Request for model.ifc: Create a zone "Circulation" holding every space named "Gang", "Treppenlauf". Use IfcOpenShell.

First a look at what the model holds.

```python
import ifcopenshell

model = ifcopenshell.open("model.ifc")
print(model.schema)
seen = {}
for space in model.by_type("IfcSpace"):
    seen[space.LongName] = seen.get(space.LongName, 0) + 1
for name, count in sorted(seen.items(), key=str):
    print(count, "x", name)
print("zones:", [z.Name for z in model.by_type("IfcZone")][:20])
```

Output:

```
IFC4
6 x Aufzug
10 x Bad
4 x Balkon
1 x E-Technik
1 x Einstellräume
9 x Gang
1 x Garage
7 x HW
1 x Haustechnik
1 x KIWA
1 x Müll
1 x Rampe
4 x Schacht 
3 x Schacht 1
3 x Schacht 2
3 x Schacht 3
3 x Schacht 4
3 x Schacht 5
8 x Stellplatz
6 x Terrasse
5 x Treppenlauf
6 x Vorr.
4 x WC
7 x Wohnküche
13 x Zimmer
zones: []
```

```python
import ifcopenshell
import ifcopenshell.api.group
import ifcopenshell.api.root

model = ifcopenshell.open("model.ifc")

names = {"Gang", "Treppenlauf"}
spaces = [s for s in model.by_type("IfcSpace") if s.LongName in names]

zone = ifcopenshell.api.root.create_entity(model, ifc_class="IfcZone", name="Circulation")
ifcopenshell.api.group.assign_group(model, products=spaces, group=zone)
print(len(spaces), "spaces in", zone.Name)

model.write("model_updated.ifc")
```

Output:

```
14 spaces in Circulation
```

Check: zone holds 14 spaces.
